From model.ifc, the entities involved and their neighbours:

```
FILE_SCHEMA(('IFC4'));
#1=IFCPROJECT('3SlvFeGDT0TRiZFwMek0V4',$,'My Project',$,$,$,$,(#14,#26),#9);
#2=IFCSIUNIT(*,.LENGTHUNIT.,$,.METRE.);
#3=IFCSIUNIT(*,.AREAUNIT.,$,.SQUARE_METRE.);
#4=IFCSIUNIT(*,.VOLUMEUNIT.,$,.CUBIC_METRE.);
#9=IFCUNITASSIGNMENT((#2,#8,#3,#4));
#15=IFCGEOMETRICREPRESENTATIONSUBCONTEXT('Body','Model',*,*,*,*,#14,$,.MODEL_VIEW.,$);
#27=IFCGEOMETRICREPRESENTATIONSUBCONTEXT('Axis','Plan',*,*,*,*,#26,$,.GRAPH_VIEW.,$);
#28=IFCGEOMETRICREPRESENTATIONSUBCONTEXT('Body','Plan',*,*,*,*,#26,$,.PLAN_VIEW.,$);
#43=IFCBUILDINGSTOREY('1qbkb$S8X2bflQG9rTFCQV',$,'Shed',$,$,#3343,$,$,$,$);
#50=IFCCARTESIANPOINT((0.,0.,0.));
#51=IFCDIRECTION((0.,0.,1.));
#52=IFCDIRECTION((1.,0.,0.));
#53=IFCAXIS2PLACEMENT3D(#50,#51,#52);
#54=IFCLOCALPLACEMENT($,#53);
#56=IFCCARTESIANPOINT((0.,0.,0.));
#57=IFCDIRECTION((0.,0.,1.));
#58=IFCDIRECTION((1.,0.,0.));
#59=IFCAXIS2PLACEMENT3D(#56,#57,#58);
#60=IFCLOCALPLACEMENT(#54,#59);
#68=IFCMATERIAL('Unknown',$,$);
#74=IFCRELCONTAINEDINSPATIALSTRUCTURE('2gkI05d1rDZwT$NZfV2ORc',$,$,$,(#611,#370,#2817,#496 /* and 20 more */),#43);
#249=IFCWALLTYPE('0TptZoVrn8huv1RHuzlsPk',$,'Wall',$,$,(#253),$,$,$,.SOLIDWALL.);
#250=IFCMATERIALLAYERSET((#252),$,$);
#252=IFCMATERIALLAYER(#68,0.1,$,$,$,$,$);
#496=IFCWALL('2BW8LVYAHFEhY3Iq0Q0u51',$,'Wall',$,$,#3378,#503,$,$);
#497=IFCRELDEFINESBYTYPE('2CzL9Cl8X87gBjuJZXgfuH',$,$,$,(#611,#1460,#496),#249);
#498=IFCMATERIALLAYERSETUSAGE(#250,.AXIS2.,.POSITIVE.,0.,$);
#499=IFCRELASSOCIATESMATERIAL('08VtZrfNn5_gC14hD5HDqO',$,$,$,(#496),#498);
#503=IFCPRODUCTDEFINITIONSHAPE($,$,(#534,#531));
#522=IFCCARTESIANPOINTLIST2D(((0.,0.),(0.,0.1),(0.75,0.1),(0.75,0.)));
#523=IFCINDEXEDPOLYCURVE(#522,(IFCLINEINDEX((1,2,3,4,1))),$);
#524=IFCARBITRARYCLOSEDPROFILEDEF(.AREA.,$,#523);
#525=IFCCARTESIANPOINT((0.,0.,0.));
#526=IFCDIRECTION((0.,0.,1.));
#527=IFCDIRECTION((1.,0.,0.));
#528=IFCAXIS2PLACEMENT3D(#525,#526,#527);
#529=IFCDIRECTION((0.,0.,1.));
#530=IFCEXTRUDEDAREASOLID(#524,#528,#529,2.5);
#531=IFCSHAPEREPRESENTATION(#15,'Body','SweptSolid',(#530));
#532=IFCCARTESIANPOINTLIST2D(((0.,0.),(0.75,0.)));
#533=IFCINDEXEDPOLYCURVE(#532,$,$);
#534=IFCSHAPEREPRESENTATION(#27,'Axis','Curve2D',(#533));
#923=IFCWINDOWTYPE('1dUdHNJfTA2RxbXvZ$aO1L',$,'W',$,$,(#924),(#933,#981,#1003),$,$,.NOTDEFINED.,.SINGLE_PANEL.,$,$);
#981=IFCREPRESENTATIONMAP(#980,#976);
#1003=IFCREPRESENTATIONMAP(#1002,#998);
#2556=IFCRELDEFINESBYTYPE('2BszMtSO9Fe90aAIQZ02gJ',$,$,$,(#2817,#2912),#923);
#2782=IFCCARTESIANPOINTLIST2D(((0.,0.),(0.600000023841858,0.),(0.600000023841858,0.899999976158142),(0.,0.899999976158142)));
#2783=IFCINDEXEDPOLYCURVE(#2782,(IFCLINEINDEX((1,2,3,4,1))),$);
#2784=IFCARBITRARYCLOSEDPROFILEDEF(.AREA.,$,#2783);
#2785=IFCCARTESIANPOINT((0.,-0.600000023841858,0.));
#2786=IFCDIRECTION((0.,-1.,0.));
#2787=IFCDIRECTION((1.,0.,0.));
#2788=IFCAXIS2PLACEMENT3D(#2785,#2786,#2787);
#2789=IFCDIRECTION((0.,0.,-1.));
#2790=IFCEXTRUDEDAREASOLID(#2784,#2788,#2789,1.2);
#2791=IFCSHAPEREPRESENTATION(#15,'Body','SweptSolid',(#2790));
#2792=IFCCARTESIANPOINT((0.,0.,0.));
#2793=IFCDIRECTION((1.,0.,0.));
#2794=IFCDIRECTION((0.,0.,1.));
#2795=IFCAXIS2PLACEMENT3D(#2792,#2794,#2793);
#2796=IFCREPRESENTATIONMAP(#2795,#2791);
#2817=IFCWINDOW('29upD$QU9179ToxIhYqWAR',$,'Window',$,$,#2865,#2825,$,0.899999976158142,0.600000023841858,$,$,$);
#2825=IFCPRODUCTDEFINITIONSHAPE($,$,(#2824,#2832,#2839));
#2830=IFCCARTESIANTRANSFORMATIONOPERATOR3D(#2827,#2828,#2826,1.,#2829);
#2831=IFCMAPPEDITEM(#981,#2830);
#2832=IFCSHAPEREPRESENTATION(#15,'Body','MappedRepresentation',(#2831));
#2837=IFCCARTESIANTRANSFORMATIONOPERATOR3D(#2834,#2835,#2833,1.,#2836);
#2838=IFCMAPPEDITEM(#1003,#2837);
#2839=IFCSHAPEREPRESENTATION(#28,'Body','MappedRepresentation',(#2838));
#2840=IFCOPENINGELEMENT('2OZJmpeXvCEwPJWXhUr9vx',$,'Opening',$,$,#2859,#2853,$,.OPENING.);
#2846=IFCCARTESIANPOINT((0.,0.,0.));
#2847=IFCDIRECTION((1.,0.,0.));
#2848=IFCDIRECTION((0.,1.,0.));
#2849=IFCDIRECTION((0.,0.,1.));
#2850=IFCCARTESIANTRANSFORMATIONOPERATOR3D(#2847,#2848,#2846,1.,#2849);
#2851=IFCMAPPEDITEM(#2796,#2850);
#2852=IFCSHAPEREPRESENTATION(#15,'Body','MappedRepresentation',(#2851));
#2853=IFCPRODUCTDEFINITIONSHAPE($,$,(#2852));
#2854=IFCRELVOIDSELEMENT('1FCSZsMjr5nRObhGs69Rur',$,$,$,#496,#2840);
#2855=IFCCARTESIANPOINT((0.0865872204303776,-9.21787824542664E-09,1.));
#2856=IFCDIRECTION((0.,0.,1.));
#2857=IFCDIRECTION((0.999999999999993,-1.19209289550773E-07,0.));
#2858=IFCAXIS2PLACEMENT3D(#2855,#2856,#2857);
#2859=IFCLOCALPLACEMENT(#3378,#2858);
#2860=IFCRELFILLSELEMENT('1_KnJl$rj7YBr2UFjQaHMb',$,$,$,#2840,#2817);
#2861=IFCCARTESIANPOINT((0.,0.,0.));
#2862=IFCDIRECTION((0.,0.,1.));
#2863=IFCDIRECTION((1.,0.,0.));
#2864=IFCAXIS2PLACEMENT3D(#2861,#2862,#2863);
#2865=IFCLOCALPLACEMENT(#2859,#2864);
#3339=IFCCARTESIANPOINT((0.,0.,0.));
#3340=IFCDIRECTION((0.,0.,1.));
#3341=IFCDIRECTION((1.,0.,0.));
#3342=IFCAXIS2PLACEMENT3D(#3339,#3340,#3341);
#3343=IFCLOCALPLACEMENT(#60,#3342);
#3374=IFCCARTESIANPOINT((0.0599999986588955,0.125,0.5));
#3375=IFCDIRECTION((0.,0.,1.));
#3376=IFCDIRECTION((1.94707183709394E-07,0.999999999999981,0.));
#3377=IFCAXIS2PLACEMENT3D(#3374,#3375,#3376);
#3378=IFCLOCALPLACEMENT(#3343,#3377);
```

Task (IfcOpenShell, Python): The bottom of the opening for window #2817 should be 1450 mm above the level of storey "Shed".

```python
import numpy as np
import ifcopenshell
import ifcopenshell.api.geometry
import ifcopenshell.geom
import ifcopenshell.util.element
import ifcopenshell.util.placement
import ifcopenshell.util.shape
import ifcopenshell.util.unit

model = ifcopenshell.open("model.ifc")
unit_scale = ifcopenshell.util.unit.calculate_unit_scale(model)

window = model.by_id(2817)
opening = window.FillsVoids[0].RelatingOpeningElement
storey = ifcopenshell.util.element.get_container(window, ifc_class="IfcBuildingStorey")
level = ifcopenshell.util.placement.get_local_placement(storey.ObjectPlacement)[2, 3]

# The opening's origin need not be at the sill, so measure its lowest point.
shape = ifcopenshell.geom.create_shape(ifcopenshell.geom.settings(), opening)
bottom = ifcopenshell.util.shape.get_shape_bottom_elevation(shape, shape.geometry) / unit_scale
dz = level + 1.45 / unit_scale - bottom

shift = np.array([0.0, 0.0, dz])
# The window is placed relative to its opening, so it follows when the opening moves.
matrix = ifcopenshell.util.placement.get_local_placement(opening.ObjectPlacement)
matrix[:3, 3] += shift
ifcopenshell.api.geometry.edit_object_placement(
    model, product=opening, matrix=matrix, is_si=False, should_transform_children=True
)

print(f"moved by {dz * unit_scale:+.3f} m")

model.write("model_updated.ifc")
```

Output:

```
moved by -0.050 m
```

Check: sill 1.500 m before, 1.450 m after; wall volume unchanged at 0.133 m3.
